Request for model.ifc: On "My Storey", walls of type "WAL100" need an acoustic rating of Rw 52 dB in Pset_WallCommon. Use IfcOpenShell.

First a look at what the model holds.

```python
import ifcopenshell
import ifcopenshell.util.element

model = ifcopenshell.open("model.ifc")
print(model.schema)
storey = next(s for s in model.by_type("IfcBuildingStorey") if s.Name == "My Storey")
walls = [e for e in ifcopenshell.util.element.get_decomposition(storey) if e.is_a("IfcWall")]
seen = {}
for e in walls:
    element_type = ifcopenshell.util.element.get_type(e)
    key = (element_type.Name if element_type != e and element_type else None, ifcopenshell.util.element.get_pset(e, "Pset_WallCommon", "AcousticRating"))
    seen[key] = seen.get(key, 0) + 1
for (name, value), count in sorted(seen.items(), key=str):
    print(count, "x", name, "|", value)
```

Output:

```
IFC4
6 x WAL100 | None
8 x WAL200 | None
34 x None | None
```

```python
import ifcopenshell
import ifcopenshell.api.pset
import ifcopenshell.util.element

model = ifcopenshell.open("model.ifc")

storey = next(s for s in model.by_type("IfcBuildingStorey") if s.Name == "My Storey")
walls = [e for e in ifcopenshell.util.element.get_decomposition(storey) if e.is_a("IfcWall")]

count = 0
for e in walls:
    element_type = ifcopenshell.util.element.get_type(e)
    if element_type in (None, e) or element_type.Name != "WAL100":
        continue
    # add_pset returns the element's existing set when there is one.
    pset = ifcopenshell.api.pset.add_pset(model, product=e, name="Pset_WallCommon")
    ifcopenshell.api.pset.edit_pset(model, pset=pset, properties={"AcousticRating": "Rw 52 dB"})
    count += 1

print(count, "walls updated")

model.write("model-out.ifc")
```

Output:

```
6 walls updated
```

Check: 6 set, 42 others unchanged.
